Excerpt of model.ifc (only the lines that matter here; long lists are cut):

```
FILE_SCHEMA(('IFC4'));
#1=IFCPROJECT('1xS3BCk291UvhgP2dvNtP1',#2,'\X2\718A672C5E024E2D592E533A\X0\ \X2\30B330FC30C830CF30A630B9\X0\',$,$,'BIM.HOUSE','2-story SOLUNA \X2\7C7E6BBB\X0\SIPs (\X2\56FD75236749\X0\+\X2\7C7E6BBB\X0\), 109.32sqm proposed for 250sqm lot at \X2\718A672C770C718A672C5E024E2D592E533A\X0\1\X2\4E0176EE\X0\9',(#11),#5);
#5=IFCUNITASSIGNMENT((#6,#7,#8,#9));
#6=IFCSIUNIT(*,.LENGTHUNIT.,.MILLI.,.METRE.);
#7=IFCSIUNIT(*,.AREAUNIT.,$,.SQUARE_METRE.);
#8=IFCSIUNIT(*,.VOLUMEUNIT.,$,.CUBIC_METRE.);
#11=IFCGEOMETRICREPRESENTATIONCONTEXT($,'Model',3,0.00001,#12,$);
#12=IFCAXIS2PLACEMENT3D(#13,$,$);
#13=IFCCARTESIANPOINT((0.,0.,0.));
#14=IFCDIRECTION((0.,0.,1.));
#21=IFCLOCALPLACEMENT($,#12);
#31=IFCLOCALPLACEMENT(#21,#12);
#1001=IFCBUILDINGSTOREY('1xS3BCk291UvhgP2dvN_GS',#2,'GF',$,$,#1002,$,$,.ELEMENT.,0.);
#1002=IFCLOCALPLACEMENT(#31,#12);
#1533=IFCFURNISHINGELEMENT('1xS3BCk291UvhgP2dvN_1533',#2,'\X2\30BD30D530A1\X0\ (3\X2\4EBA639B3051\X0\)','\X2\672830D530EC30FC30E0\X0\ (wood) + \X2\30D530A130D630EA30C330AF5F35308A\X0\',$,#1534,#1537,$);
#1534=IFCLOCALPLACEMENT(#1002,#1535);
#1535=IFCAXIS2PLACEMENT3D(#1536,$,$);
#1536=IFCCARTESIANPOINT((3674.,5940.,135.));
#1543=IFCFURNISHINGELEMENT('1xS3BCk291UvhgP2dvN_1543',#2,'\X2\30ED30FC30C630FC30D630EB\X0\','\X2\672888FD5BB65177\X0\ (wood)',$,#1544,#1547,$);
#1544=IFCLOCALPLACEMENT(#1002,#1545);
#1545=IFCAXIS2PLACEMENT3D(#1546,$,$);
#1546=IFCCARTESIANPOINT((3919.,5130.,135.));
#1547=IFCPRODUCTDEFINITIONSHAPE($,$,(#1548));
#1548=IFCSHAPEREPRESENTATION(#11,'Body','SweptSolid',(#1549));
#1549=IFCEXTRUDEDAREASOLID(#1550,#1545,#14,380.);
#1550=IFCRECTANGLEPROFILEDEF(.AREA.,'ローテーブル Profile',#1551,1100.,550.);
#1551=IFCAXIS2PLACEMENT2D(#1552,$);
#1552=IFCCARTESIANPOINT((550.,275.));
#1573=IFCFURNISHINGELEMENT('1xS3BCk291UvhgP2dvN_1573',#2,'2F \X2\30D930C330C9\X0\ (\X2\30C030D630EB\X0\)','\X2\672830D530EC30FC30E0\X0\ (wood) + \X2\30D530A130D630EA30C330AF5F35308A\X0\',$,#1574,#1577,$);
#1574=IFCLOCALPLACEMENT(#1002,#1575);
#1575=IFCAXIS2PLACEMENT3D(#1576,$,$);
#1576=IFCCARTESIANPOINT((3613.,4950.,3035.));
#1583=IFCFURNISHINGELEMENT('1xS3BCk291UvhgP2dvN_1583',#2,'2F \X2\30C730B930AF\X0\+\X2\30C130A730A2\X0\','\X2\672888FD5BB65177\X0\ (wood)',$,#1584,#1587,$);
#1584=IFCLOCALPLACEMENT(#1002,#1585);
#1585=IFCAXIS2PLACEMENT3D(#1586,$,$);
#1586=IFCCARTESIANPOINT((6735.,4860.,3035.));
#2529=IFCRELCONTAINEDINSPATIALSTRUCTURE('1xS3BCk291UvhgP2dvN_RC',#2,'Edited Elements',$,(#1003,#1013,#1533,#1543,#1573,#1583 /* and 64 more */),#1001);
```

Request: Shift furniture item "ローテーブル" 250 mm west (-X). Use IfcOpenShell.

```python
import ifcopenshell
import ifcopenshell.api.geometry
import ifcopenshell.util.placement

model = ifcopenshell.open("model.ifc")

item = model.by_id(1543)
matrix = ifcopenshell.util.placement.get_local_placement(item.ObjectPlacement)
matrix[0, 3] -= 250.0
ifcopenshell.api.geometry.edit_object_placement(model, product=item, matrix=matrix, is_si=False)

print(ifcopenshell.util.placement.get_local_placement(item.ObjectPlacement).round(3) + 0.0)

model.write("model-out.ifc")
```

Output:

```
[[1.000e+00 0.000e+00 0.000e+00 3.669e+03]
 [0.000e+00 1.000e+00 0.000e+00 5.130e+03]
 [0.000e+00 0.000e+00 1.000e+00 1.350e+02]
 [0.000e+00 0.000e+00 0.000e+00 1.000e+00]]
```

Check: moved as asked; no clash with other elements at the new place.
